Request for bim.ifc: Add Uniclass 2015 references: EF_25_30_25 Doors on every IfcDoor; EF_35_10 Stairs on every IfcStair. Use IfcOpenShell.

First a look at what the model holds.

```python
import ifcopenshell

model = ifcopenshell.open("bim.ifc")
print(model.schema)
print("classifications:", [c.Name for c in model.by_type("IfcClassification")])
for ifc_class in ("IfcDoor", "IfcRoof", "IfcStair", "IfcWall", "IfcWindow"):
    print(ifc_class, len(model.by_type(ifc_class)))
```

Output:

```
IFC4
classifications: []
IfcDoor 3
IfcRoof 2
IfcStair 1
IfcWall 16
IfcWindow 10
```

```python
import ifcopenshell
import ifcopenshell.api.classification

model = ifcopenshell.open("bim.ifc")

system = ifcopenshell.api.classification.add_classification(model, classification="Uniclass 2015")

codes = {
    "IfcDoor": ("EF_25_30_25", "Doors"),
    "IfcStair": ("EF_35_10", "Stairs"),
}
for ifc_class, (code, name) in codes.items():
    products = model.by_type(ifc_class)
    ifcopenshell.api.classification.add_reference(
        model, products=products, classification=system, identification=code, name=name
    )
    print(code, len(products))

model.write("bim_v2.ifc")
```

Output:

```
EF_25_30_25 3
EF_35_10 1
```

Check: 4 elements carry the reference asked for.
